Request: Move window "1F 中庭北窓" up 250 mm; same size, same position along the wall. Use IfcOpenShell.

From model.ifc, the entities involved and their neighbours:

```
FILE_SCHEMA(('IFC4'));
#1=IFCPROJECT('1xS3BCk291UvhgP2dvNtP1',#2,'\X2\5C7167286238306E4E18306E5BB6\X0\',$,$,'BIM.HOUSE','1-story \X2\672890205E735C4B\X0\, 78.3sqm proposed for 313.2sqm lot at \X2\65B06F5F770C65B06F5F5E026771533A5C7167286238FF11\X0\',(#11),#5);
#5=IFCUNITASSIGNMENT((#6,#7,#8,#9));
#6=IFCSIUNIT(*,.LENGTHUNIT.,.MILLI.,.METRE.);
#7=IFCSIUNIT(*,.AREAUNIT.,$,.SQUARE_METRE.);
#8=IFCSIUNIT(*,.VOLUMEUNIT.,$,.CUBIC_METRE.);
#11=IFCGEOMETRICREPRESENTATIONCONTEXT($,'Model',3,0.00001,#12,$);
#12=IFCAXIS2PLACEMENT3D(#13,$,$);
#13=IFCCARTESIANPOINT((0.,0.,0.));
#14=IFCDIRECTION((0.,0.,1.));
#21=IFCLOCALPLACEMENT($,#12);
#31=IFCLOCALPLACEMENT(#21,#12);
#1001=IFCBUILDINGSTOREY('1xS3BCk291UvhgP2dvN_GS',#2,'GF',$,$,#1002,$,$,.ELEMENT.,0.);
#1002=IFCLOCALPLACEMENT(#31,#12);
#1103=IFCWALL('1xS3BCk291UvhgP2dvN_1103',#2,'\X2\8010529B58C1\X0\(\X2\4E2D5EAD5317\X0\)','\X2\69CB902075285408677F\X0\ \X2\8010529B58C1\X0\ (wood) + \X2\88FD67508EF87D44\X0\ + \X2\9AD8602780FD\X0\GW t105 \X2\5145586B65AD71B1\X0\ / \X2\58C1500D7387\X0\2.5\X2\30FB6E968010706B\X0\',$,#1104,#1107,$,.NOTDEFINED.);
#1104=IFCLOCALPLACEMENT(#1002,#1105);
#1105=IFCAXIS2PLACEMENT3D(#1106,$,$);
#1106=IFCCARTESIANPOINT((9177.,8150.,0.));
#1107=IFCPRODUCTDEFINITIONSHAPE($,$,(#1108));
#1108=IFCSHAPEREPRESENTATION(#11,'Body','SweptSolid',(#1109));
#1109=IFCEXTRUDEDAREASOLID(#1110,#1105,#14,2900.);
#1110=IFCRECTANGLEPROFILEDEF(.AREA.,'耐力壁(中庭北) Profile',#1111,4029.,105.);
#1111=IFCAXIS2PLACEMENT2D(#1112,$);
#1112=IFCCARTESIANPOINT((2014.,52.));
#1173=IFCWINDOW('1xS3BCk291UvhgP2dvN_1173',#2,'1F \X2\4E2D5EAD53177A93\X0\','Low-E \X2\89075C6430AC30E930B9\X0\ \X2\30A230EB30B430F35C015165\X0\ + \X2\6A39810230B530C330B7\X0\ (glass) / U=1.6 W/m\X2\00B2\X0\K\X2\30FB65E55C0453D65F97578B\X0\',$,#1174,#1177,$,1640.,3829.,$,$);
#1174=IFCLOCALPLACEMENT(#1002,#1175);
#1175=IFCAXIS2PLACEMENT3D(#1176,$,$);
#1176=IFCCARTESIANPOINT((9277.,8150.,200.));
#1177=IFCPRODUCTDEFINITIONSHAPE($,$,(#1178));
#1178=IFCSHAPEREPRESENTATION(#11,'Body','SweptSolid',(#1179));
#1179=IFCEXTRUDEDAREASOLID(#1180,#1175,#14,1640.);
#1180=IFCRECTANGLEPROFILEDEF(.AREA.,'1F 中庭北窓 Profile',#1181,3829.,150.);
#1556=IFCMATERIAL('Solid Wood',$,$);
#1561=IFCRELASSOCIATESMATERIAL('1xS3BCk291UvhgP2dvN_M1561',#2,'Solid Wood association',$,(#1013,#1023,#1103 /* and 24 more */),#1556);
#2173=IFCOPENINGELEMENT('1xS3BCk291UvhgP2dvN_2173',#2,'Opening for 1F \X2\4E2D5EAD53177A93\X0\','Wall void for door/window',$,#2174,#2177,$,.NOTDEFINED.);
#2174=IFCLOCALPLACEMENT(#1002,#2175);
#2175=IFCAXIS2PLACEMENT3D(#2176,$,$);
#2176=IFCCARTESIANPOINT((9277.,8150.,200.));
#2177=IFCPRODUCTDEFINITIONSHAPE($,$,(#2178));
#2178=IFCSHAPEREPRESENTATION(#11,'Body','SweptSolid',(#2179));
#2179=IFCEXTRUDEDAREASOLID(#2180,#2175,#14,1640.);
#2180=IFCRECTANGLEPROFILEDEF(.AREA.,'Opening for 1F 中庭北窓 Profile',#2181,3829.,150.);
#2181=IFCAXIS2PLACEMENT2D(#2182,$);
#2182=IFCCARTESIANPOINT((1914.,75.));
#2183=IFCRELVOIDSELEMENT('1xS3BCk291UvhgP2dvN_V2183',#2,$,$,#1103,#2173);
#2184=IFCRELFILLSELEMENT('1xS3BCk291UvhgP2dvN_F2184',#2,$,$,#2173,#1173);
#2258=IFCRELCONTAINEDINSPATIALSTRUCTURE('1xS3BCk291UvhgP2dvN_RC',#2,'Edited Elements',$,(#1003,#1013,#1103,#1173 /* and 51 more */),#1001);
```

```python
import numpy as np
import ifcopenshell
import ifcopenshell.api.geometry
import ifcopenshell.util.placement
import ifcopenshell.util.unit

model = ifcopenshell.open("model.ifc")
unit_scale = ifcopenshell.util.unit.calculate_unit_scale(model)

window = model.by_guid("1xS3BCk291UvhgP2dvN_1173")
opening = window.FillsVoids[0].RelatingOpeningElement
dz = 250.0

shift = np.array([0.0, 0.0, dz])
# The window is not placed relative to its opening, so move both.
for product in (opening, window):
    matrix = ifcopenshell.util.placement.get_local_placement(product.ObjectPlacement)
    matrix[:3, 3] += shift
    ifcopenshell.api.geometry.edit_object_placement(model, product=product, matrix=matrix, is_si=False)

print(f"moved by {dz * unit_scale:+.3f} m")

model.write("model_edited.ifc")
```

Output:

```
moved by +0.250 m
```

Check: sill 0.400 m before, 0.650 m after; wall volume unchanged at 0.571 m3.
